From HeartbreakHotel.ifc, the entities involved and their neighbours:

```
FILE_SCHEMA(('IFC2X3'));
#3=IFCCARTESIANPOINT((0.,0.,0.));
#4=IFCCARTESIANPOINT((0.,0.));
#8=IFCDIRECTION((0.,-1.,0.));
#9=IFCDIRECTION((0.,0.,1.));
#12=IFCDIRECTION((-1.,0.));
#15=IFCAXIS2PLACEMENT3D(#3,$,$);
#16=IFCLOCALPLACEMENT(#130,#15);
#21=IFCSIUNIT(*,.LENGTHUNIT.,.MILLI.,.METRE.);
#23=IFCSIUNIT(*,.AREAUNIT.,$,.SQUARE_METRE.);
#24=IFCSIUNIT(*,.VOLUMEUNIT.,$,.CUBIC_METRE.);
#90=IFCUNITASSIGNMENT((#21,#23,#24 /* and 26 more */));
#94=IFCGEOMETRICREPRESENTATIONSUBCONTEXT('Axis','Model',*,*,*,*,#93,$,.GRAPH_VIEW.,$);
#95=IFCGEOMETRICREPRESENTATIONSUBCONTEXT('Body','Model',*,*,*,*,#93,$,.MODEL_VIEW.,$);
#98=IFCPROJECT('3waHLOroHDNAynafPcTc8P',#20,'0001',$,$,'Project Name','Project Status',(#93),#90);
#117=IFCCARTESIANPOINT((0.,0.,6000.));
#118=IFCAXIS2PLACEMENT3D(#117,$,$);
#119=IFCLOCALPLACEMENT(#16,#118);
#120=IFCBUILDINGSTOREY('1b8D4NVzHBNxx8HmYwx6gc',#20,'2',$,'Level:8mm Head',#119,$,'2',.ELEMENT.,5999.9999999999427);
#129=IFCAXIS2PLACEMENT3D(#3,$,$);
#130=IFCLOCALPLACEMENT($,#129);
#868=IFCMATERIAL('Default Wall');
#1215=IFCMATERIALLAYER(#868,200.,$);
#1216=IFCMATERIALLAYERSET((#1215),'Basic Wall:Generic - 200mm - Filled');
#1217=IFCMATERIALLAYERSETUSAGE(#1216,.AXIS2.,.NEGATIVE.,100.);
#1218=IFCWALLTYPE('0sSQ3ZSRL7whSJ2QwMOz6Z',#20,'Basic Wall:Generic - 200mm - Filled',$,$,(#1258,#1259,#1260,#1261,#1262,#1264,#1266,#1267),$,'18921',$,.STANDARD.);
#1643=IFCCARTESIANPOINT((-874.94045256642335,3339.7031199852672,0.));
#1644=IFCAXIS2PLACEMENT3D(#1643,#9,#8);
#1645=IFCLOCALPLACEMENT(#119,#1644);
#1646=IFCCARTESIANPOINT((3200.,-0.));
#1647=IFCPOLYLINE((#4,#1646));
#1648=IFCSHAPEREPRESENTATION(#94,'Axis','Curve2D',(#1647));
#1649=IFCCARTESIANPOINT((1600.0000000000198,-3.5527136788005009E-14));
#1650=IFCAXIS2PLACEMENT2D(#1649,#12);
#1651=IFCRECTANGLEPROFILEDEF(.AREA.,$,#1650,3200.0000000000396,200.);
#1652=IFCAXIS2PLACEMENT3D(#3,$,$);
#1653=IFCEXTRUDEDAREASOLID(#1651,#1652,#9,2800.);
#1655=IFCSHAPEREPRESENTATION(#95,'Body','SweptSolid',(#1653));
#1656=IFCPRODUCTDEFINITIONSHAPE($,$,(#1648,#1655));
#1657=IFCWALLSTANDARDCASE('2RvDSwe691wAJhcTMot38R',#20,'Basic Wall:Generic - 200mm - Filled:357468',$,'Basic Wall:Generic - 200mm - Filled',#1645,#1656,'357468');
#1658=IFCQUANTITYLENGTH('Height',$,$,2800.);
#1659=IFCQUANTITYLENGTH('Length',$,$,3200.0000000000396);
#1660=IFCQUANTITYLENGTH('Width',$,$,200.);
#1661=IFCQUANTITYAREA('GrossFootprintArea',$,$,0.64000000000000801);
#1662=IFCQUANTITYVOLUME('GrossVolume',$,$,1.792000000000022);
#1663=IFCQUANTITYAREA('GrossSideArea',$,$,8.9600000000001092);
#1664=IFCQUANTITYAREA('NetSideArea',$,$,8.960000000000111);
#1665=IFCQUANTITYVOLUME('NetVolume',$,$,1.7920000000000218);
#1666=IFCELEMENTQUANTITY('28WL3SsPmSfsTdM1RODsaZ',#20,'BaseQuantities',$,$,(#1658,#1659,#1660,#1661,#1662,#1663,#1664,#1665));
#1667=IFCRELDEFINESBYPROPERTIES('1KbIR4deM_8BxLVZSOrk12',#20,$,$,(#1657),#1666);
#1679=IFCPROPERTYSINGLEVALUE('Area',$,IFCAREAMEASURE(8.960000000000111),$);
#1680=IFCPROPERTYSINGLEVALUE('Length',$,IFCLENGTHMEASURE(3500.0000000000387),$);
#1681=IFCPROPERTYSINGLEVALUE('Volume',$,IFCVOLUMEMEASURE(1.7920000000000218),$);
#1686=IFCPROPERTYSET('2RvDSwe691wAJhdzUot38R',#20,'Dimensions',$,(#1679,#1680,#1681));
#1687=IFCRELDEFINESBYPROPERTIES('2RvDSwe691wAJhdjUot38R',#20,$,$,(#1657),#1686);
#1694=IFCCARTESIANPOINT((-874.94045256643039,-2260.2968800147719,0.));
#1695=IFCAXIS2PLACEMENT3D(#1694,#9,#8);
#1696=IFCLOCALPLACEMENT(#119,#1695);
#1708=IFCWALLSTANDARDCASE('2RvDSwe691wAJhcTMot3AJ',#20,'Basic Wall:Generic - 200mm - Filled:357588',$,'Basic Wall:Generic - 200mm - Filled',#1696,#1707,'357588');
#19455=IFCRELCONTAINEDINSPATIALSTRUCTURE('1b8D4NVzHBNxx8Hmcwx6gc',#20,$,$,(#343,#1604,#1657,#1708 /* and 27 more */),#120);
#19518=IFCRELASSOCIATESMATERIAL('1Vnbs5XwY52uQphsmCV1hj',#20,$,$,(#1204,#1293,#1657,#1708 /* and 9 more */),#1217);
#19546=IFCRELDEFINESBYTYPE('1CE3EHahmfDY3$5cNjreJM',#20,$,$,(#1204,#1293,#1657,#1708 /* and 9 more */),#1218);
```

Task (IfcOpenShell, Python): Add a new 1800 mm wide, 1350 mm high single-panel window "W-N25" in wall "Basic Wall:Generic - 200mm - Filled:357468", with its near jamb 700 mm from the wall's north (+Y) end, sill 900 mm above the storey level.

```python
import numpy as np
import ifcopenshell
import ifcopenshell.api.feature
import ifcopenshell.api.geometry
import ifcopenshell.api.pset
import ifcopenshell.api.root
import ifcopenshell.api.spatial
import ifcopenshell.api.type
import ifcopenshell.geom
import ifcopenshell.util.element
import ifcopenshell.util.placement
import ifcopenshell.util.representation
import ifcopenshell.util.shape
import ifcopenshell.util.unit

model = ifcopenshell.open("HeartbreakHotel.ifc")
unit_scale = ifcopenshell.util.unit.calculate_unit_scale(model)
area_scale = ifcopenshell.util.unit.calculate_unit_scale(model, "AREAUNIT")
volume_scale = ifcopenshell.util.unit.calculate_unit_scale(model, "VOLUMEUNIT")
settings = ifcopenshell.geom.settings()


def volume(element):
    """Net volume in cubic metres, openings subtracted."""
    shape = ifcopenshell.geom.create_shape(settings, element)
    return ifcopenshell.util.shape.get_volume(shape.geometry)


wall = model.by_id(1657)
storey = ifcopenshell.util.element.get_container(wall, ifc_class="IfcBuildingStorey")
context = ifcopenshell.util.representation.get_context(model, "Model", "Body", "MODEL_VIEW")
before = volume(wall)

width, height, from_end, sill = 1.8, 1.35, 0.7, 0.9  # metres

# The wall runs along its own X axis, and the end named is its -X end.
wall_shape = ifcopenshell.geom.create_shape(settings, wall)
x, y, z = ifcopenshell.util.shape.get_vertices(wall_shape.geometry).T
start = x.min() + from_end
face, thickness = float(y.min()), float(y.max() - y.min())
wall_matrix = ifcopenshell.util.placement.get_local_placement(wall.ObjectPlacement)
level = ifcopenshell.util.placement.get_local_placement(storey.ObjectPlacement)[2, 3]


def in_wall(x, y):
    """Placement at x, y metres in the wall's axes, at sill height."""
    matrix = wall_matrix.copy()
    matrix[:, 3] = wall_matrix @ np.array([x / unit_scale, y / unit_scale, 0.0, 1.0])
    matrix[2, 3] = level + sill / unit_scale
    return matrix


# Opening: a box that overshoots both wall faces by 50 mm.
opening = ifcopenshell.api.root.create_entity(model, ifc_class="IfcOpeningElement")
box = ifcopenshell.api.geometry.add_wall_representation(
    model, context=context, length=width, height=height, thickness=thickness + 0.1
)
ifcopenshell.api.geometry.assign_representation(model, product=opening, representation=box)
ifcopenshell.api.geometry.edit_object_placement(model, product=opening, matrix=in_wall(start, face - 0.05), is_si=False)
ifcopenshell.api.feature.add_feature(model, feature=opening, element=wall)

window = ifcopenshell.api.root.create_entity(model, ifc_class="IfcWindow", name="W-N25")
window.OverallWidth, window.OverallHeight = width / unit_scale, height / unit_scale
body = ifcopenshell.api.geometry.add_window_representation(
    model,
    context=context,
    overall_width=window.OverallWidth,
    overall_height=window.OverallHeight,
    partition_type="SINGLE_PANEL",
)
ifcopenshell.api.geometry.assign_representation(model, product=window, representation=body)
ifcopenshell.api.spatial.assign_container(model, products=[window], relating_structure=storey)
fills = ifcopenshell.api.feature.add_filling(model, opening=opening, element=window)
fills.OwnerHistory = window.OwnerHistory  # required in IFC2X3

# IFC2X3 keeps the operation on the window style.
style = ifcopenshell.api.root.create_entity(model, ifc_class="IfcWindowStyle", name="W-N25")
style.OperationType, style.ConstructionType = "SINGLE_PANEL", "NOTDEFINED"
style.ParameterTakesPrecedence = style.Sizeable = False
ifcopenshell.api.type.assign_type(model, related_objects=[window], relating_type=style)

# Centre the window in the wall's thickness.
ifcopenshell.api.geometry.edit_object_placement(model, product=window, matrix=in_wall(start, face), is_si=False)
window_shape = ifcopenshell.geom.create_shape(settings, window)
depth = ifcopenshell.util.shape.get_vertices(window_shape.geometry)[:, 1]
offset = face + thickness / 2 - (depth.min() + depth.max()) / 2
ifcopenshell.api.geometry.edit_object_placement(model, product=window, matrix=in_wall(start, offset), is_si=False)

after = volume(wall)

# Update the wall's stored quantities.
qto = model.by_id(ifcopenshell.util.element.get_pset(wall, "BaseQuantities", should_inherit=False)["id"])
ifcopenshell.api.pset.edit_qto(model, qto=qto, properties={
    "NetSideArea": after / thickness / area_scale,
    "NetVolume": after / volume_scale,
})
pset = model.by_id(ifcopenshell.util.element.get_pset(wall, "Dimensions", should_inherit=False)["id"])
ifcopenshell.api.pset.edit_pset(model, pset=pset, properties={
    "Area": model.create_entity("IfcAreaMeasure", after / thickness / area_scale),
    "Volume": model.create_entity("IfcVolumeMeasure", after / volume_scale),
})

print(f"wall volume {before:.3f} -> {after:.3f} m3")

model.write("HeartbreakHotel_updated.ifc")
```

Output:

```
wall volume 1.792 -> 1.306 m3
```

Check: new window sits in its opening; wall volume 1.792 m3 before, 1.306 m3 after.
